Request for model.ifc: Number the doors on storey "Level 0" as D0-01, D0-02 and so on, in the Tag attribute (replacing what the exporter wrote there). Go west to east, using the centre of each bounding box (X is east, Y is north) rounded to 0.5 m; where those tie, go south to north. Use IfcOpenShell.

First a look at what the model holds.

```python
import ifcopenshell
import ifcopenshell.util.element
import ifcopenshell.util.placement

model = ifcopenshell.open("model.ifc")
print(model.schema)
storey = next(s for s in model.by_type("IfcBuildingStorey") if s.Name == "Level 0")
doors = [e for e in ifcopenshell.util.element.get_decomposition(storey) if e.is_a("IfcDoor")]
for e in sorted(doors, key=lambda e: e.id()):
    origin = ifcopenshell.util.placement.get_local_placement(e.ObjectPlacement)[:3, 3]
    print(e.id(), e.Tag, e.Name, origin.round(2) + 0.0, sep=" | ")
```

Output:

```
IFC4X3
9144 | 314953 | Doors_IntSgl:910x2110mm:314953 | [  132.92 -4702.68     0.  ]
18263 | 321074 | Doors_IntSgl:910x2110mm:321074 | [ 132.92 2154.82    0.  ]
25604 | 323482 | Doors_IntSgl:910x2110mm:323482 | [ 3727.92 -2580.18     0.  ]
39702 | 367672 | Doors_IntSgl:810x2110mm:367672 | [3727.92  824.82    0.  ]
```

```python
import ifcopenshell
import ifcopenshell.geom
import ifcopenshell.util.element
import ifcopenshell.util.shape

model = ifcopenshell.open("model.ifc")
settings = ifcopenshell.geom.settings()
settings.set("use-world-coords", True)


def centre(element):
    shape = ifcopenshell.geom.create_shape(settings, element)
    return ifcopenshell.util.shape.get_bbox_centroid(shape.geometry)


storey = next(s for s in model.by_type("IfcBuildingStorey") if s.Name == "Level 0")
doors = [e for e in ifcopenshell.util.element.get_decomposition(storey) if e.is_a("IfcDoor")]

# Insertion points can sit at a corner or the storey origin, so sort by the geometry (in metres).
centres = {e: centre(e) for e in doors}
doors.sort(key=lambda e: (round(centres[e][0] / 0.5), centres[e][1]))

for i, e in enumerate(doors, start=1):
    number = f"D0-{i:02d}"
    e.Tag = number
    print(e.id(), number)

model.write("model_updated.ifc")
```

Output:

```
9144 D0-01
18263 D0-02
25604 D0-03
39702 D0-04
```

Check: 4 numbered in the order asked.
